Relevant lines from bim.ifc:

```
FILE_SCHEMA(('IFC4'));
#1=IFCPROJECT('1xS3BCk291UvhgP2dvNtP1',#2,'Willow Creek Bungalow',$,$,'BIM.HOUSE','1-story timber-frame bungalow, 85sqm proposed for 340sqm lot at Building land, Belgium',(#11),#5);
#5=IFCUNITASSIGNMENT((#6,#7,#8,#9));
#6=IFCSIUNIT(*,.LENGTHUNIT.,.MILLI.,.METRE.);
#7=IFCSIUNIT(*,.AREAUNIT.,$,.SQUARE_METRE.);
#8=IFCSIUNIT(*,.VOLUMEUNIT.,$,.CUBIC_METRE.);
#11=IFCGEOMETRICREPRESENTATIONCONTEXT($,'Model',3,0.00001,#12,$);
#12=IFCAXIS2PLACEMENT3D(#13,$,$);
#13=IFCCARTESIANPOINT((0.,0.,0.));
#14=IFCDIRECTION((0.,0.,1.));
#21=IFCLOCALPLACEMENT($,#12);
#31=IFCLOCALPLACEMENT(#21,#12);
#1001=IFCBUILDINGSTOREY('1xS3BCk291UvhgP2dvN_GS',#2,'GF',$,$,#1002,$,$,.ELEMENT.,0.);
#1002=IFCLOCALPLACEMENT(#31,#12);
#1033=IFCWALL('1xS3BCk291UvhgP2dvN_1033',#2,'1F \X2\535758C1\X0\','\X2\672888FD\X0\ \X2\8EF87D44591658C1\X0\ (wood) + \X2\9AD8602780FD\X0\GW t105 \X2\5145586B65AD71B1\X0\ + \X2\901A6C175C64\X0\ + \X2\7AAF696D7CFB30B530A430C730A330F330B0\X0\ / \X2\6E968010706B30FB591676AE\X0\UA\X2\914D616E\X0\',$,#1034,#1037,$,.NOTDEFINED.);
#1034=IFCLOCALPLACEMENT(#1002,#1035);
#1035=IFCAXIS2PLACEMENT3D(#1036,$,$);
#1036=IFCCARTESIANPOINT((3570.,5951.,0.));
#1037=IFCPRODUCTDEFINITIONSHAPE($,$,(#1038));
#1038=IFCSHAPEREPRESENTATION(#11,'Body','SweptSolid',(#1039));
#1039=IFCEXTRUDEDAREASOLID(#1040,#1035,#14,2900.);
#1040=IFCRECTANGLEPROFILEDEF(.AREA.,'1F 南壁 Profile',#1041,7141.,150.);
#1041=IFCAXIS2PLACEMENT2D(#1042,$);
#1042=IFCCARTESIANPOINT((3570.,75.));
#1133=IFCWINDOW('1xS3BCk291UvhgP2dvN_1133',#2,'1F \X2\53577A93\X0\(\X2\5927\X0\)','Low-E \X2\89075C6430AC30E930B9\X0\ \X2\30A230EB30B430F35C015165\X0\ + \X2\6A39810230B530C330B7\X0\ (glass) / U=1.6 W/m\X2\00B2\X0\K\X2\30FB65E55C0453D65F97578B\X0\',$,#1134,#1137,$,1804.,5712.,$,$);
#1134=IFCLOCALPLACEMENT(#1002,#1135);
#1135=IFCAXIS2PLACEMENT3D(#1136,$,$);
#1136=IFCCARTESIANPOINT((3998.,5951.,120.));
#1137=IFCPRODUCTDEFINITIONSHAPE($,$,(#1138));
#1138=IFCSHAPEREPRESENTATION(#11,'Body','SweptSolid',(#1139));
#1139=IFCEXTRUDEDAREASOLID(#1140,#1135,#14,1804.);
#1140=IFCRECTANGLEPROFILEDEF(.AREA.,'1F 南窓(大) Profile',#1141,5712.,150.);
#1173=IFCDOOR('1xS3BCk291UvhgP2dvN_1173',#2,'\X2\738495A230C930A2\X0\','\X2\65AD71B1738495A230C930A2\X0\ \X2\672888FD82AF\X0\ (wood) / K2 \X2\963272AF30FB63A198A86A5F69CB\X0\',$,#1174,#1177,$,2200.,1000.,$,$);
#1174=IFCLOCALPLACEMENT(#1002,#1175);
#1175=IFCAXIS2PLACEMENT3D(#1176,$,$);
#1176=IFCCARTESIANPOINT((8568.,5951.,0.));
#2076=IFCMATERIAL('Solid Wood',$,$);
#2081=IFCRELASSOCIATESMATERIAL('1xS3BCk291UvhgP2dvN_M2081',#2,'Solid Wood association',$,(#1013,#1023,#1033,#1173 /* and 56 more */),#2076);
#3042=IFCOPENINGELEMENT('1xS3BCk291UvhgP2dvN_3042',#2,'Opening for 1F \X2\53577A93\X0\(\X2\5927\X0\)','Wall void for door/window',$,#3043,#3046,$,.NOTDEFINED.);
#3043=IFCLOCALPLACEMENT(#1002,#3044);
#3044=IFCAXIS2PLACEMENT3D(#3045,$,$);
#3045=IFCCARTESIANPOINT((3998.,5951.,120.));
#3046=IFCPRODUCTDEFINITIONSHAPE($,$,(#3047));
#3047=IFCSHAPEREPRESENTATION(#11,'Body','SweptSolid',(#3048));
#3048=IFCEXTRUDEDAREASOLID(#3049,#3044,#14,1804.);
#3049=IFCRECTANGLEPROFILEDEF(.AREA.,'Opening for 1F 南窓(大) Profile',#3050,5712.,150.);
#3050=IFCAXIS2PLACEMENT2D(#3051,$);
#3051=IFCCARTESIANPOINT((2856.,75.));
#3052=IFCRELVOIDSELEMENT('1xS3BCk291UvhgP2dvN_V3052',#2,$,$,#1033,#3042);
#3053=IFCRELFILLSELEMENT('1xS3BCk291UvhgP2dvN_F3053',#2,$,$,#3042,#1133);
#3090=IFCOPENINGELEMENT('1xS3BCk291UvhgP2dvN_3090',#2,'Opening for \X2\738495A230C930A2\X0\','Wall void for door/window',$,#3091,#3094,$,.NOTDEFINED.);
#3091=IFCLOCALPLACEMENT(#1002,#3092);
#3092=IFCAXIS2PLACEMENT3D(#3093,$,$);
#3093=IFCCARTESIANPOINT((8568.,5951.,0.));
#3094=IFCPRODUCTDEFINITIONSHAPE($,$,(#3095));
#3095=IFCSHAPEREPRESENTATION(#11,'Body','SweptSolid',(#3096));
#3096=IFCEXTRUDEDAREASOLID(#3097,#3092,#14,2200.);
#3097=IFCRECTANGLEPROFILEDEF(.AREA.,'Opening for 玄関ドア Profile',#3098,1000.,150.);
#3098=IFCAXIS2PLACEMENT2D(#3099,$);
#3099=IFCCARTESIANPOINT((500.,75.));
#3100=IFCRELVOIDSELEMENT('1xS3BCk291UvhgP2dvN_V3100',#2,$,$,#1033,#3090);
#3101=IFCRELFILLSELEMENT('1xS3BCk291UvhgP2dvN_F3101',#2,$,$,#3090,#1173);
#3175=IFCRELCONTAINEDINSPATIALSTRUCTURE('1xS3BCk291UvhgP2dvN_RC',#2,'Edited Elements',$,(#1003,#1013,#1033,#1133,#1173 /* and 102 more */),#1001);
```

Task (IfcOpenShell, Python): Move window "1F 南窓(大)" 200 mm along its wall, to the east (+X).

```python
import ifcopenshell
import ifcopenshell.api.geometry
import ifcopenshell.util.placement
import ifcopenshell.util.unit

model = ifcopenshell.open("bim.ifc")
unit_scale = ifcopenshell.util.unit.calculate_unit_scale(model)

window = model.by_guid("1xS3BCk291UvhgP2dvN_1133")
opening = window.FillsVoids[0].RelatingOpeningElement
wall = opening.VoidsElements[0].RelatingBuildingElement

wall_matrix = ifcopenshell.util.placement.get_local_placement(wall.ObjectPlacement)
shift = wall_matrix[:3, 0] * 0.2 / unit_scale
before = ifcopenshell.util.placement.get_local_placement(window.ObjectPlacement)[:3, 3].copy()

# The window is not placed relative to its opening, so move both.
for product in (opening, window):
    matrix = ifcopenshell.util.placement.get_local_placement(product.ObjectPlacement)
    matrix[:3, 3] += shift
    ifcopenshell.api.geometry.edit_object_placement(model, product=product, matrix=matrix, is_si=False)

after = ifcopenshell.util.placement.get_local_placement(window.ObjectPlacement)[:3, 3]
print("window moved by", (after - before).round(3) + 0.0)

model.write("bim_edited.ifc")
```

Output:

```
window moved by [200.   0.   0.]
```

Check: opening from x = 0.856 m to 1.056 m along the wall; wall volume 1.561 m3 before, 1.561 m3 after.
